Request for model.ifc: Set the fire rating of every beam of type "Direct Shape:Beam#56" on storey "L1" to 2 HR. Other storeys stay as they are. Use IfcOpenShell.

First a look at what the model holds.

```python
import ifcopenshell
import ifcopenshell.util.element

model = ifcopenshell.open("model.ifc")
print(model.schema)
storey = next(s for s in model.by_type("IfcBuildingStorey") if s.Name == "L1")
beams = [e for e in ifcopenshell.util.element.get_decomposition(storey) if e.is_a("IfcBeam")]
seen = {}
for e in beams:
    element_type = ifcopenshell.util.element.get_type(e)
    key = (element_type.Name if element_type != e and element_type else None, ifcopenshell.util.element.get_pset(e, "Pset_BeamCommon", "FireRating"))
    seen[key] = seen.get(key, 0) + 1
for (name, value), count in sorted(seen.items(), key=str):
    print(count, "x", name, "|", value)
```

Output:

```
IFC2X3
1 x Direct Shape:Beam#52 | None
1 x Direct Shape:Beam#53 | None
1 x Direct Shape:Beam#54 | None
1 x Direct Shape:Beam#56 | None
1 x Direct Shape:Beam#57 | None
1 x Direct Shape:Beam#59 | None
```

```python
import ifcopenshell
import ifcopenshell.api.pset
import ifcopenshell.util.element

model = ifcopenshell.open("model.ifc")

storey = next(s for s in model.by_type("IfcBuildingStorey") if s.Name == "L1")
beams = [e for e in ifcopenshell.util.element.get_decomposition(storey) if e.is_a("IfcBeam")]

count = 0
for e in beams:
    element_type = ifcopenshell.util.element.get_type(e)
    if element_type in (None, e) or element_type.Name != "Direct Shape:Beam#56":
        continue
    # add_pset returns the element's existing set when there is one.
    pset = ifcopenshell.api.pset.add_pset(model, product=e, name="Pset_BeamCommon")
    ifcopenshell.api.pset.edit_pset(model, pset=pset, properties={"FireRating": "2 HR"})
    count += 1

print(count, "beams updated")

model.write("model_rev.ifc")
```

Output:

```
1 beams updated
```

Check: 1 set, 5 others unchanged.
